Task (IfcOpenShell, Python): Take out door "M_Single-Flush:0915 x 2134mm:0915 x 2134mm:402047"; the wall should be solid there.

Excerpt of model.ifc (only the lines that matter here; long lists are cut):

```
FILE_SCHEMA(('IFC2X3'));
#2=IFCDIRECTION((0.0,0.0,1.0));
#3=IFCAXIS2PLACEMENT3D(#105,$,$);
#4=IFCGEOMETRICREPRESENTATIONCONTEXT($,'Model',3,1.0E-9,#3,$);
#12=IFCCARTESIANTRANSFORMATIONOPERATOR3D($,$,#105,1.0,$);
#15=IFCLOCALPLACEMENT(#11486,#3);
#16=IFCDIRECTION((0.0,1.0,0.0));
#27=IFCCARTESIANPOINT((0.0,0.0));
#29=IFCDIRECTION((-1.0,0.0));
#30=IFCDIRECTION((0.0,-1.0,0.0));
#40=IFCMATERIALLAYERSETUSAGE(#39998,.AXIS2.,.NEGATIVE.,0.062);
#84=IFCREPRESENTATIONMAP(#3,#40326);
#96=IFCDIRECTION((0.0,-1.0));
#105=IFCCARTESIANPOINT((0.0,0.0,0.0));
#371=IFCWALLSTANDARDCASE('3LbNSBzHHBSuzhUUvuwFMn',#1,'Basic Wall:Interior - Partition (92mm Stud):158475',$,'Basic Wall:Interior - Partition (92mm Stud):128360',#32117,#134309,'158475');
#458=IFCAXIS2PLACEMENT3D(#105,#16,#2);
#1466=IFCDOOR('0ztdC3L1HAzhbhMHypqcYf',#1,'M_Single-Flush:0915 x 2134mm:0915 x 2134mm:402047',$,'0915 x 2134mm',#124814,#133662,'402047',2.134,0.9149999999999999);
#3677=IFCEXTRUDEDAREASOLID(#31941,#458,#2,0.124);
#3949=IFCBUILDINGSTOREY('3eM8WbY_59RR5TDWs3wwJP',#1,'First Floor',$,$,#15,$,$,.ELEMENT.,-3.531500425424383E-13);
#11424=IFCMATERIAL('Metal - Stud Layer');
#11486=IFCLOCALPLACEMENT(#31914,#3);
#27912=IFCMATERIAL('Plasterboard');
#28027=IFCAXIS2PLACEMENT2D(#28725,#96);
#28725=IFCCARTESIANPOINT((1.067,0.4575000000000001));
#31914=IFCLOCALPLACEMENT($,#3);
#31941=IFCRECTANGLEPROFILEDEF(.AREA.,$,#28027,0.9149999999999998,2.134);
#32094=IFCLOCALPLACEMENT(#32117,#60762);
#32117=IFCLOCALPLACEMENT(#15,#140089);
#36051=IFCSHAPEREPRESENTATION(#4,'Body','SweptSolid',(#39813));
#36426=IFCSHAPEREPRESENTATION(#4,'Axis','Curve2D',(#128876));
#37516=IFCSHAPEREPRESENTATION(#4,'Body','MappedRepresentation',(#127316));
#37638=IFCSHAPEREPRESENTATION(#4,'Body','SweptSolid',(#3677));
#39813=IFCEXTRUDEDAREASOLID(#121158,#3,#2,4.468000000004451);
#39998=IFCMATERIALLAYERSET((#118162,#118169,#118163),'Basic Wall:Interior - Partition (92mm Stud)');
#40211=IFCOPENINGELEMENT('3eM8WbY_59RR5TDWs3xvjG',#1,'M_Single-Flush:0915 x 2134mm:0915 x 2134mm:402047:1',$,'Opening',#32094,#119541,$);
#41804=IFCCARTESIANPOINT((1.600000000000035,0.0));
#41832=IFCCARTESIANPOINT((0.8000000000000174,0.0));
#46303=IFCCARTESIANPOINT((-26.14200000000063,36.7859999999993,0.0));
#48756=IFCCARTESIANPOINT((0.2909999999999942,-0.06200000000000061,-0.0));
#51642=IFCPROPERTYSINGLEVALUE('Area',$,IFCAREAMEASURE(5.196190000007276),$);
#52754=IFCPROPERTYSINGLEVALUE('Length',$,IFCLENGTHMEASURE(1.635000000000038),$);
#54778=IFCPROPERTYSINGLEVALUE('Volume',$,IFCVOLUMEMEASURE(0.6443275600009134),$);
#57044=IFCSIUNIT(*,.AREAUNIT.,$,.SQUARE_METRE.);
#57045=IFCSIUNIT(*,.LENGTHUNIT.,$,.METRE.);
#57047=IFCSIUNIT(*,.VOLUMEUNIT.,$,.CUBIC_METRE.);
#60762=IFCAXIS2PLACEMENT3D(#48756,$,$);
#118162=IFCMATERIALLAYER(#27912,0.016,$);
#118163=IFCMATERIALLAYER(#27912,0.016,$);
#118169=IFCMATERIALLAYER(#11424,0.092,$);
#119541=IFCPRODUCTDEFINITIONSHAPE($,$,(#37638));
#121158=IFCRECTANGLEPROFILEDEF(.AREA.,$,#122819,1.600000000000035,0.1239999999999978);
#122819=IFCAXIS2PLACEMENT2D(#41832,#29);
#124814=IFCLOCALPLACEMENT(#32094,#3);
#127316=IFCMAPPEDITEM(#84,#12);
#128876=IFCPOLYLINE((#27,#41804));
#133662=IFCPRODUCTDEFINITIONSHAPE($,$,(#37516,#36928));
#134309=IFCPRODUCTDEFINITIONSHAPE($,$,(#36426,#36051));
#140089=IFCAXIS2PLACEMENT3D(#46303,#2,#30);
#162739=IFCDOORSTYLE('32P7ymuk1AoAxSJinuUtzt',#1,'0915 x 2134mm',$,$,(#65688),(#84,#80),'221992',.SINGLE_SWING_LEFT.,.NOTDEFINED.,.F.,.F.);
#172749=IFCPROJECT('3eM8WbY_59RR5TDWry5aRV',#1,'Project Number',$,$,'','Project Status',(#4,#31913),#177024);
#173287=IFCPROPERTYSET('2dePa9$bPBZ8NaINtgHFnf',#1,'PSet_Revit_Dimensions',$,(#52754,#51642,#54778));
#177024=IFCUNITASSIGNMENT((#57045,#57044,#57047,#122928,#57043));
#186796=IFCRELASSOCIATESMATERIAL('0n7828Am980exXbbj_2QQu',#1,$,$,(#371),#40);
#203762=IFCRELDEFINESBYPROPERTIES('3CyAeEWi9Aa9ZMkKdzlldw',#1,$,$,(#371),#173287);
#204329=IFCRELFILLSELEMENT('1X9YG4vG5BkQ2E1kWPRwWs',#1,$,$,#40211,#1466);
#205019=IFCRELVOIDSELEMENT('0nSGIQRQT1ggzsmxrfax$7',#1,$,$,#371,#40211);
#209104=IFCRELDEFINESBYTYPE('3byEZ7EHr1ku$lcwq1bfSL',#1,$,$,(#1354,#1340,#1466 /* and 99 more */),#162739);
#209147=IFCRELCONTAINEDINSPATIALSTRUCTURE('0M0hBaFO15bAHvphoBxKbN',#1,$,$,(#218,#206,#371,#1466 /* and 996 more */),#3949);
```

```python
import ifcopenshell
import ifcopenshell.api.feature
import ifcopenshell.api.pset
import ifcopenshell.api.root
import ifcopenshell.geom
import ifcopenshell.util.element
import ifcopenshell.util.shape
import ifcopenshell.util.unit

model = ifcopenshell.open("model.ifc")
area_scale = ifcopenshell.util.unit.calculate_unit_scale(model, "AREAUNIT")
volume_scale = ifcopenshell.util.unit.calculate_unit_scale(model, "VOLUMEUNIT")
settings = ifcopenshell.geom.settings()


def volume(element):
    """Net volume in cubic metres, openings subtracted."""
    shape = ifcopenshell.geom.create_shape(settings, element)
    return ifcopenshell.util.shape.get_volume(shape.geometry)


door = model.by_id(1466)
opening = door.FillsVoids[0].RelatingOpeningElement
wall = opening.VoidsElements[0].RelatingBuildingElement
before = volume(wall)

ifcopenshell.api.root.remove_product(model, product=door)
ifcopenshell.api.feature.remove_feature(model, feature=opening)

after = volume(wall)
thickness = 0.124  # wall thickness in metres

# Update the wall's stored quantities.
pset = model.by_id(ifcopenshell.util.element.get_pset(wall, "PSet_Revit_Dimensions", should_inherit=False)["id"])
ifcopenshell.api.pset.edit_pset(model, pset=pset, properties={
    "Area": model.create_entity("IfcAreaMeasure", after / thickness / area_scale),
    "Volume": model.create_entity("IfcVolumeMeasure", after / volume_scale),
})

print(f"wall volume {before:.3f} -> {after:.3f} m3")

model.write("model_edited.ifc")
```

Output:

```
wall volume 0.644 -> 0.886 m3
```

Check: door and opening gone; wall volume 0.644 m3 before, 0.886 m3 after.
